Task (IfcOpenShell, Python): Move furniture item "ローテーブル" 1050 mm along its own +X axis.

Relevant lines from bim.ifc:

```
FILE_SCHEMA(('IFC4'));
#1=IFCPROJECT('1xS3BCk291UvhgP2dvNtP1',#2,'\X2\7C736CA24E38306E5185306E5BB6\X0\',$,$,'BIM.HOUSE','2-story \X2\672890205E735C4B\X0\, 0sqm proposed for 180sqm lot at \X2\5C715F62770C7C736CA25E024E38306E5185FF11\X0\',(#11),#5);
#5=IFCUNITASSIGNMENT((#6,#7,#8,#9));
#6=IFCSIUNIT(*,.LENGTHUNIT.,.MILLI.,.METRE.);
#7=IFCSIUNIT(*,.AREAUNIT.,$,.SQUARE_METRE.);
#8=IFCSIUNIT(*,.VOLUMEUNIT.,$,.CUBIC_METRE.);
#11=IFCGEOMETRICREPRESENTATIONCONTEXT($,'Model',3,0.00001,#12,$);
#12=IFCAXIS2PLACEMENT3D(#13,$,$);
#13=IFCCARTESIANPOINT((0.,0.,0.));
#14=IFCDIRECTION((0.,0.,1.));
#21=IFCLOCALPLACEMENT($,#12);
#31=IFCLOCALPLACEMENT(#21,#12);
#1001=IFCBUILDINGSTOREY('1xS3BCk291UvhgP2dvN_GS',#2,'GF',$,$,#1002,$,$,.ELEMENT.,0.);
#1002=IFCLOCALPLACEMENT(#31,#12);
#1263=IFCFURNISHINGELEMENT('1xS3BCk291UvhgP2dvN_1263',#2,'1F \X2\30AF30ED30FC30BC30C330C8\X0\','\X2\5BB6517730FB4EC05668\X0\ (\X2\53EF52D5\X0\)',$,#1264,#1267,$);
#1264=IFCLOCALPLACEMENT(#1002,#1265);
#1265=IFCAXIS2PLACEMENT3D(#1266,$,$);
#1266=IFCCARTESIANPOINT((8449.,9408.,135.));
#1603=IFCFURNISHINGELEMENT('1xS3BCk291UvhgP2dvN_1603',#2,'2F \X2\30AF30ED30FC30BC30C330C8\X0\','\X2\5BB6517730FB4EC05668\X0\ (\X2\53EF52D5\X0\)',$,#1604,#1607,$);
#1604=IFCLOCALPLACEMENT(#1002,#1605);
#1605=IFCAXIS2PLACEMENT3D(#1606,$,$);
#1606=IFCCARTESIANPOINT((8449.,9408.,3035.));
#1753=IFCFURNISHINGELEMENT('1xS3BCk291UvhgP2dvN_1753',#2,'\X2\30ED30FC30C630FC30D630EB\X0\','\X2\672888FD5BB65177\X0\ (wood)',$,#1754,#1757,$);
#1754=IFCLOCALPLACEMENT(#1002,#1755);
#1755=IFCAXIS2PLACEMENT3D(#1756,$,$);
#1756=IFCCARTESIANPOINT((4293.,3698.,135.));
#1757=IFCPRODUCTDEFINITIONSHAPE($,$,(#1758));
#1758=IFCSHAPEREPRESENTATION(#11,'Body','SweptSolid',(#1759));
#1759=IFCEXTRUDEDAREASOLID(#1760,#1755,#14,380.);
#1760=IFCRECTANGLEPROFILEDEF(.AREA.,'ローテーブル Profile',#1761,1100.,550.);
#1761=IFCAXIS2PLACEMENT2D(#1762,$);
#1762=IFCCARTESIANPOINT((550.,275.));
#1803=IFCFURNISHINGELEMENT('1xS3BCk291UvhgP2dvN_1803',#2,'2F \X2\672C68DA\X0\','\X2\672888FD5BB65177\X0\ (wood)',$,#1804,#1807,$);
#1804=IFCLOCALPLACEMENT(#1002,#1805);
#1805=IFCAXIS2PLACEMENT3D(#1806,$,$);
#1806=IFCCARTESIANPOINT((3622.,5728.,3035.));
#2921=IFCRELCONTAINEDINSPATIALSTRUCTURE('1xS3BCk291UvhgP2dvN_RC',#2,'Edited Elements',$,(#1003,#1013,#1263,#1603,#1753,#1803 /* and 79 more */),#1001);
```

```python
import ifcopenshell
import ifcopenshell.api.geometry
import ifcopenshell.util.placement
import ifcopenshell.util.unit

model = ifcopenshell.open("bim.ifc")
unit_scale = ifcopenshell.util.unit.calculate_unit_scale(model)

item = model.by_guid("1xS3BCk291UvhgP2dvN_1753")
matrix = ifcopenshell.util.placement.get_local_placement(item.ObjectPlacement)
matrix[:3, 3] += matrix[:3, 0] * 1.05 / unit_scale
ifcopenshell.api.geometry.edit_object_placement(model, product=item, matrix=matrix, is_si=False)

print(ifcopenshell.util.placement.get_local_placement(item.ObjectPlacement).round(3) + 0.0)

model.write("bim_updated.ifc")
```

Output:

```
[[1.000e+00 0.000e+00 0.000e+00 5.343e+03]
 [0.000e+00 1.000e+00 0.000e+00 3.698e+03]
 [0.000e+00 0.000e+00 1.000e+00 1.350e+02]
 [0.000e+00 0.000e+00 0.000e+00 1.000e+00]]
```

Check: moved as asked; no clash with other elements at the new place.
